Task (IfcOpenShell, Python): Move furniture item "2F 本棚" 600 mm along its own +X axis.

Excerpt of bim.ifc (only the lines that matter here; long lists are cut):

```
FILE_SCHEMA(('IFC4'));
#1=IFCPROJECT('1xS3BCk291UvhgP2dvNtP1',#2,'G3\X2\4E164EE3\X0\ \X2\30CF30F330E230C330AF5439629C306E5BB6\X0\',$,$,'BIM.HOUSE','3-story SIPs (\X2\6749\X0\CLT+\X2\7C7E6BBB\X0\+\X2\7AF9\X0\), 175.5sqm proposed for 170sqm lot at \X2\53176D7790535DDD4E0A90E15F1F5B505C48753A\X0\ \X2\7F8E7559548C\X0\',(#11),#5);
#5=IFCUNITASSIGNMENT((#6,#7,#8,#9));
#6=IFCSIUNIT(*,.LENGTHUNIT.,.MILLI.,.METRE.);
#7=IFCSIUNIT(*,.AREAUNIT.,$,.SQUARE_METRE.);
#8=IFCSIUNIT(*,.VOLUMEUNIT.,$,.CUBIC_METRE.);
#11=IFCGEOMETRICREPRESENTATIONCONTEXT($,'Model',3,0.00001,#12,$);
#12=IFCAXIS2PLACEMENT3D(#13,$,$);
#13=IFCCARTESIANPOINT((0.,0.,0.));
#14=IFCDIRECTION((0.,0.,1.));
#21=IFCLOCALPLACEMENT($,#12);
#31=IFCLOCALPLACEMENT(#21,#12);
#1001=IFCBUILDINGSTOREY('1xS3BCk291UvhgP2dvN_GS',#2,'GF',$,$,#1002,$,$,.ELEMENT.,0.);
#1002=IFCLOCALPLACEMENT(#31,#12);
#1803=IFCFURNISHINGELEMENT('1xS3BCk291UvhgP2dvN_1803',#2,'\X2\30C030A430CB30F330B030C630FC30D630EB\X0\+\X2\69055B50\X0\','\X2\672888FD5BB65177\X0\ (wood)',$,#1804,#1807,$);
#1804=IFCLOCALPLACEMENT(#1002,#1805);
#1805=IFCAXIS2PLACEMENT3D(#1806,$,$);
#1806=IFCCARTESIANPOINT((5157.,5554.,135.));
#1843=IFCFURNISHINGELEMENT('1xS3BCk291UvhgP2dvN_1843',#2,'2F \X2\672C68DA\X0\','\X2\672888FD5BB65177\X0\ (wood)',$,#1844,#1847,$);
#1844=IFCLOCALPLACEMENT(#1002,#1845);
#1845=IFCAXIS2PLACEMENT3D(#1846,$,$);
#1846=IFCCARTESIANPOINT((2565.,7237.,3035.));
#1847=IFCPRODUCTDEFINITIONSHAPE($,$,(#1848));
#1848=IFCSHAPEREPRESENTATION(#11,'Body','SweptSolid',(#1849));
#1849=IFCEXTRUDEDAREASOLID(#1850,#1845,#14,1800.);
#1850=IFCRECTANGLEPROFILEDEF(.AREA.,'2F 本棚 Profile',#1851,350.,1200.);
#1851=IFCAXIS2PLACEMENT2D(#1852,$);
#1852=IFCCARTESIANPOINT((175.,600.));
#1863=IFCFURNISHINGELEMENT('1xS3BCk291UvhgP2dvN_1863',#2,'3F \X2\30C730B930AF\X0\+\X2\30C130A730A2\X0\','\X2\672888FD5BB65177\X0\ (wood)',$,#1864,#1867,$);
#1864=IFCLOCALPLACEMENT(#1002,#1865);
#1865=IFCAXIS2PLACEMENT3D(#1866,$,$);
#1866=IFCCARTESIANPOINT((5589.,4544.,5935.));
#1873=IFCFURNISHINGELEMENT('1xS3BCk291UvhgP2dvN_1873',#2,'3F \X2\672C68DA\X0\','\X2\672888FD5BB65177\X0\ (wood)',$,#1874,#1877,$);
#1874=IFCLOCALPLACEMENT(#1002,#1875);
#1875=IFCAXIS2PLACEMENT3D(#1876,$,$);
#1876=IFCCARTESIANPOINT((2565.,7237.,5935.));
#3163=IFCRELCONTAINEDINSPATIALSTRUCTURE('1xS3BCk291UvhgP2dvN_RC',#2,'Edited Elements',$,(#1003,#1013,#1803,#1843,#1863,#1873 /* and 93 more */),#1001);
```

```python
import ifcopenshell
import ifcopenshell.api.geometry
import ifcopenshell.util.placement
import ifcopenshell.util.unit

model = ifcopenshell.open("bim.ifc")
unit_scale = ifcopenshell.util.unit.calculate_unit_scale(model)

item = model.by_guid("1xS3BCk291UvhgP2dvN_1843")
matrix = ifcopenshell.util.placement.get_local_placement(item.ObjectPlacement)
matrix[:3, 3] += matrix[:3, 0] * 0.6 / unit_scale
ifcopenshell.api.geometry.edit_object_placement(model, product=item, matrix=matrix, is_si=False)

print(ifcopenshell.util.placement.get_local_placement(item.ObjectPlacement).round(3) + 0.0)

model.write("bim_rev.ifc")
```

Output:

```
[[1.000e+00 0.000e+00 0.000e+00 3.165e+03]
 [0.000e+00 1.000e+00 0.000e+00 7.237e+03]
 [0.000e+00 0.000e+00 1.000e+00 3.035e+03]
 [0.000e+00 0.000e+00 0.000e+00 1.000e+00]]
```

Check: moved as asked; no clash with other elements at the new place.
